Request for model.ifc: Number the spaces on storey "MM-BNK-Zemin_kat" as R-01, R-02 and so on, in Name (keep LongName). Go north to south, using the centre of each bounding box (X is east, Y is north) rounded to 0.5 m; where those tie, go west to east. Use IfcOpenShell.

First a look at what the model holds.

```python
import ifcopenshell
import ifcopenshell.util.element
import ifcopenshell.util.placement

model = ifcopenshell.open("model.ifc")
print(model.schema)
storey = next(s for s in model.by_type("IfcBuildingStorey") if s.Name == "MM-BNK-Zemin_kat")
spaces = [e for e in ifcopenshell.util.element.get_decomposition(storey) if e.is_a("IfcSpace")]
for e in sorted(spaces, key=lambda e: e.id()):
    origin = ifcopenshell.util.placement.get_local_placement(e.ObjectPlacement)[:3, 3]
    print(e.id(), e.Name, e.LongName, origin.round(2) + 0.0, sep=" | ")
```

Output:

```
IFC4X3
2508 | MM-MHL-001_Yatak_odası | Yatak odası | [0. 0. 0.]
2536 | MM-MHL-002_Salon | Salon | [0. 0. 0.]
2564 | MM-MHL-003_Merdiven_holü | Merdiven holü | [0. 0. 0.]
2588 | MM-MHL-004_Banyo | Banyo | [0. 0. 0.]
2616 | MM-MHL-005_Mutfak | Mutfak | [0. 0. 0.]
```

```python
import ifcopenshell
import ifcopenshell.geom
import ifcopenshell.util.element
import ifcopenshell.util.shape

model = ifcopenshell.open("model.ifc")
settings = ifcopenshell.geom.settings()
settings.set("use-world-coords", True)


def centre(element):
    shape = ifcopenshell.geom.create_shape(settings, element)
    return ifcopenshell.util.shape.get_bbox_centroid(shape.geometry)


storey = next(s for s in model.by_type("IfcBuildingStorey") if s.Name == "MM-BNK-Zemin_kat")
spaces = [e for e in ifcopenshell.util.element.get_decomposition(storey) if e.is_a("IfcSpace")]

# Insertion points can sit at a corner or the storey origin, so sort by the geometry (in metres).
centres = {e: centre(e) for e in spaces}
spaces.sort(key=lambda e: (-round(centres[e][1] / 0.5), centres[e][0]))

for i, e in enumerate(spaces, start=1):
    number = f"R-{i:02d}"
    e.Name = number
    print(e.id(), number)

model.write("model-out.ifc")
```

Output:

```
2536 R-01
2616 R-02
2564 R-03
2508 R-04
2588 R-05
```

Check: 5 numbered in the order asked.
